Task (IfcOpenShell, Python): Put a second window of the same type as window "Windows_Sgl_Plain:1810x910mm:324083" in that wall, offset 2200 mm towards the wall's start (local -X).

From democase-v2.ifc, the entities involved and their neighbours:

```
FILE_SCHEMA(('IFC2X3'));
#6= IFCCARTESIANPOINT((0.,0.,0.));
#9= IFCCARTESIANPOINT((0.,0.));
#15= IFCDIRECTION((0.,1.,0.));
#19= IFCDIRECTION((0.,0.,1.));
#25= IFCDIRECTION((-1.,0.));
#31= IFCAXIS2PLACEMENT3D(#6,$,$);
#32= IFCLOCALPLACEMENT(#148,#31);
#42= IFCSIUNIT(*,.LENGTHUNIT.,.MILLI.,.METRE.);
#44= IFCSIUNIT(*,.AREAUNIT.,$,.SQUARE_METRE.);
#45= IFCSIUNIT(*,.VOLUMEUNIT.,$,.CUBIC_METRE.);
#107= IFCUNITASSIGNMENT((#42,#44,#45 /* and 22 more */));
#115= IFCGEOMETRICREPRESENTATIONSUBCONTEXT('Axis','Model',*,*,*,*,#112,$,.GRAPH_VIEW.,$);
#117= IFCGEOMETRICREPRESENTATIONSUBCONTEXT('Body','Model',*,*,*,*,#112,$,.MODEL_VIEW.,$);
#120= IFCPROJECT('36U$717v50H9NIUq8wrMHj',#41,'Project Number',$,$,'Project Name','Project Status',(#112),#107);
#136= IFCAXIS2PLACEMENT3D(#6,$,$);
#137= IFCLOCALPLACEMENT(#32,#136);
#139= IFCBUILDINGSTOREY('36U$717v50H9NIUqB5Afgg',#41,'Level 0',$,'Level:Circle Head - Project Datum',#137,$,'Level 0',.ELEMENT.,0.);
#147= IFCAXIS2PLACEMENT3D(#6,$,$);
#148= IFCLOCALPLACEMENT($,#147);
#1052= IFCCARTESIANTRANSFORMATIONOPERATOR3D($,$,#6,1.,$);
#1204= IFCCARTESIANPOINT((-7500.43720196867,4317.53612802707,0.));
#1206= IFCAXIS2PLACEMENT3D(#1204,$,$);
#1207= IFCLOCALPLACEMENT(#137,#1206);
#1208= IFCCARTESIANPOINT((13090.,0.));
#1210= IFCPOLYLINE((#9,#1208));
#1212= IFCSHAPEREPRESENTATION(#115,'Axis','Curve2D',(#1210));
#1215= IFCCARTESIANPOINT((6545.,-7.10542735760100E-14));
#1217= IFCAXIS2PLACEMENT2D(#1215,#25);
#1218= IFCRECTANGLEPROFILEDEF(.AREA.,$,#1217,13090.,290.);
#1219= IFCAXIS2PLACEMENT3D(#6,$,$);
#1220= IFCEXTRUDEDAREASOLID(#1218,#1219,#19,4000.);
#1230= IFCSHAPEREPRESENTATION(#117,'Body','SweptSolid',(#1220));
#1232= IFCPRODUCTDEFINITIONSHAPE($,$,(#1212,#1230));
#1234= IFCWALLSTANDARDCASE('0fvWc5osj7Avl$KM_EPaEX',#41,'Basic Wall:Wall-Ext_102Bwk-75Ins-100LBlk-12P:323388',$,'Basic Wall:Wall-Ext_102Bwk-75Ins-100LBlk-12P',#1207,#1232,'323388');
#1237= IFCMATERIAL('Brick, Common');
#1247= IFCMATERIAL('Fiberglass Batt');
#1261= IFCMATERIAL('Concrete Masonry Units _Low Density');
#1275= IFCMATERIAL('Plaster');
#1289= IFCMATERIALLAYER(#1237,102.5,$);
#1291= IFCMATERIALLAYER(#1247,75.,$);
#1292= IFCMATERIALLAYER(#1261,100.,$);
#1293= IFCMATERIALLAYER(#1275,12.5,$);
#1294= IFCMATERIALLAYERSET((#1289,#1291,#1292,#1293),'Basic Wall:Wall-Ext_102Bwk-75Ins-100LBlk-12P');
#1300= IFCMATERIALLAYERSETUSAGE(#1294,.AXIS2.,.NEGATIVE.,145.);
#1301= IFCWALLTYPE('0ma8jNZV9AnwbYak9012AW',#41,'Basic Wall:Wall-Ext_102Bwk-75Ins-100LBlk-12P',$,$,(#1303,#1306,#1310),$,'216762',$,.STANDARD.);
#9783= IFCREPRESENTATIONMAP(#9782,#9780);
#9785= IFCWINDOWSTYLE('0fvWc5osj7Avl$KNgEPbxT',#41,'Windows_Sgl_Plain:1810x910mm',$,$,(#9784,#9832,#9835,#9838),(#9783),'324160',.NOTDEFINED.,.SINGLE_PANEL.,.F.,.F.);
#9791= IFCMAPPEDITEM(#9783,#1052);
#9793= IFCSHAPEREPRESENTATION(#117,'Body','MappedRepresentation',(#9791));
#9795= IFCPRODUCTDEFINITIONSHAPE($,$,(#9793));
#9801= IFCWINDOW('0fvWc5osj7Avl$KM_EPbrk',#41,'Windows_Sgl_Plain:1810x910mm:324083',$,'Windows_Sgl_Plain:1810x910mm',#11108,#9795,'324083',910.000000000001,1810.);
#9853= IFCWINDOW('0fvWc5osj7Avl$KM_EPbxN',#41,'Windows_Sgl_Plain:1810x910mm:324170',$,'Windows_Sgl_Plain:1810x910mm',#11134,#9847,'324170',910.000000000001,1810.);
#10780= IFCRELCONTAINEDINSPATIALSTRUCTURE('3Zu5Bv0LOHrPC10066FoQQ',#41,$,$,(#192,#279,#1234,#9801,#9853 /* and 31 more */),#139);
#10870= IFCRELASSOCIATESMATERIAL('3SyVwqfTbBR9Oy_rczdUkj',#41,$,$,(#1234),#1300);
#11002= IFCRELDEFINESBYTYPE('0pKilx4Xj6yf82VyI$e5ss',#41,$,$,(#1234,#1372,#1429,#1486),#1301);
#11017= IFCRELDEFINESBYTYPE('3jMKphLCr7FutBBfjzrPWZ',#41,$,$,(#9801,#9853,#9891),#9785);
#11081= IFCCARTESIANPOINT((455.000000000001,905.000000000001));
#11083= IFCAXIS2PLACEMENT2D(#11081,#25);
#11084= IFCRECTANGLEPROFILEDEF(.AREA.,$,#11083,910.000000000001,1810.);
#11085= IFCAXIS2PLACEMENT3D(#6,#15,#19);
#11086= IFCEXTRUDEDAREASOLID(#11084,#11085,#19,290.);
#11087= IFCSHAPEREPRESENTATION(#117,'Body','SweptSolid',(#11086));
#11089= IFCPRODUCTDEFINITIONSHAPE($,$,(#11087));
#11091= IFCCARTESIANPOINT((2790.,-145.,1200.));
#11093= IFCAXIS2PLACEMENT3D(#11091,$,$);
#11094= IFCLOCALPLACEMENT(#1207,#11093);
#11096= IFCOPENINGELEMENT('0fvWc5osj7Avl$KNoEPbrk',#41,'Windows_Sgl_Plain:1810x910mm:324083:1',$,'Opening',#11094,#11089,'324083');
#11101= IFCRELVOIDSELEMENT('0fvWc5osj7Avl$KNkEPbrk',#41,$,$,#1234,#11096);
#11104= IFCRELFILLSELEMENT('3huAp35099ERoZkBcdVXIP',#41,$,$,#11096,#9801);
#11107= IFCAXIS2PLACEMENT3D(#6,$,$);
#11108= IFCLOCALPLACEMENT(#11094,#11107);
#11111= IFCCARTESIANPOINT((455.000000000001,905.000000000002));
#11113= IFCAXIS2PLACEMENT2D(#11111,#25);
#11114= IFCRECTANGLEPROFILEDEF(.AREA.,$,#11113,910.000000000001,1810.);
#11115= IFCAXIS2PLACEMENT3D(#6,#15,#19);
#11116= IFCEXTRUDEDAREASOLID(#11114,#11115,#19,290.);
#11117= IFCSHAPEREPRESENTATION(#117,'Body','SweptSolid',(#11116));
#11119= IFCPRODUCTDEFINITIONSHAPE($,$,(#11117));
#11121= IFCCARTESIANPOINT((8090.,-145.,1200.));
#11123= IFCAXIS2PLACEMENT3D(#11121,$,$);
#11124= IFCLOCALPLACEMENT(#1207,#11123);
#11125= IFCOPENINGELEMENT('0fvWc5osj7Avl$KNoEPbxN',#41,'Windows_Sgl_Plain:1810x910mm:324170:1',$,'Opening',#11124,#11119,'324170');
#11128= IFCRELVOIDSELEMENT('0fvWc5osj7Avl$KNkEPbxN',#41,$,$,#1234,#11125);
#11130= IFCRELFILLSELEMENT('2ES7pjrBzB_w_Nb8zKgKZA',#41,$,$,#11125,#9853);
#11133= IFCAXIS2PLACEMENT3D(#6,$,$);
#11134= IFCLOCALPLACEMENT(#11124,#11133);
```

```python
import ifcopenshell
import ifcopenshell.api.feature
import ifcopenshell.api.geometry
import ifcopenshell.api.root
import ifcopenshell.geom
import ifcopenshell.util.element
import ifcopenshell.util.placement
import ifcopenshell.util.shape
import ifcopenshell.util.unit

model = ifcopenshell.open("democase-v2.ifc")
unit_scale = ifcopenshell.util.unit.calculate_unit_scale(model)
settings = ifcopenshell.geom.settings()


def volume(element):
    """Net volume in cubic metres, openings subtracted."""
    shape = ifcopenshell.geom.create_shape(settings, element)
    return ifcopenshell.util.shape.get_volume(shape.geometry)


def reuse_history(source, copy):
    """copy_class also copies each property set's owner history, people and application; keep the originals."""
    for rel in copy.IsDefinedBy:
        if rel.is_a("IfcRelDefinesByProperties") and (history := rel.RelatingPropertyDefinition.OwnerHistory):
            rel.RelatingPropertyDefinition.OwnerHistory = source.OwnerHistory
            ifcopenshell.util.element.remove_deep2(model, history)


window = model.by_guid("0fvWc5osj7Avl$KM_EPbrk")
opening = window.FillsVoids[0].RelatingOpeningElement
wall = opening.VoidsElements[0].RelatingBuildingElement
before = volume(wall)
shift = ifcopenshell.util.placement.get_local_placement(wall.ObjectPlacement)[:3, 0] * -2.2 / unit_scale

# copy_class copies the void relationship, type, container and properties, but no geometry.
new_opening = ifcopenshell.api.root.copy_class(model, product=opening)
new_opening.Representation = ifcopenshell.util.element.copy_deep(
    model, opening.Representation, exclude=["IfcGeometricRepresentationContext", "IfcRepresentationMap"]
)
new_opening.Name = "Windows_Sgl_Plain:1810x910mm"
new_opening.Tag = None
new_window = ifcopenshell.api.root.copy_class(model, product=window)
new_window.Representation = ifcopenshell.util.element.copy_deep(
    model, window.Representation, exclude=["IfcGeometricRepresentationContext", "IfcRepresentationMap"]
)
new_window.Name = "Windows_Sgl_Plain:1810x910mm"
new_window.Tag = None
reuse_history(window, new_window)
fills = ifcopenshell.api.feature.add_filling(model, opening=new_opening, element=new_window)
fills.OwnerHistory = new_window.OwnerHistory  # required in IFC2X3

for old, new in ((opening, new_opening), (window, new_window)):
    matrix = ifcopenshell.util.placement.get_local_placement(old.ObjectPlacement)
    matrix[:3, 3] += shift
    ifcopenshell.api.geometry.edit_object_placement(model, product=new, matrix=matrix, is_si=False)

after = volume(wall)

print(f"wall volume {before:.3f} -> {after:.3f} m3")

model.write("democase-v2_edited.ifc")
```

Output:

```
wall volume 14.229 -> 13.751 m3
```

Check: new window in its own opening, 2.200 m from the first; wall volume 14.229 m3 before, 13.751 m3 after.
